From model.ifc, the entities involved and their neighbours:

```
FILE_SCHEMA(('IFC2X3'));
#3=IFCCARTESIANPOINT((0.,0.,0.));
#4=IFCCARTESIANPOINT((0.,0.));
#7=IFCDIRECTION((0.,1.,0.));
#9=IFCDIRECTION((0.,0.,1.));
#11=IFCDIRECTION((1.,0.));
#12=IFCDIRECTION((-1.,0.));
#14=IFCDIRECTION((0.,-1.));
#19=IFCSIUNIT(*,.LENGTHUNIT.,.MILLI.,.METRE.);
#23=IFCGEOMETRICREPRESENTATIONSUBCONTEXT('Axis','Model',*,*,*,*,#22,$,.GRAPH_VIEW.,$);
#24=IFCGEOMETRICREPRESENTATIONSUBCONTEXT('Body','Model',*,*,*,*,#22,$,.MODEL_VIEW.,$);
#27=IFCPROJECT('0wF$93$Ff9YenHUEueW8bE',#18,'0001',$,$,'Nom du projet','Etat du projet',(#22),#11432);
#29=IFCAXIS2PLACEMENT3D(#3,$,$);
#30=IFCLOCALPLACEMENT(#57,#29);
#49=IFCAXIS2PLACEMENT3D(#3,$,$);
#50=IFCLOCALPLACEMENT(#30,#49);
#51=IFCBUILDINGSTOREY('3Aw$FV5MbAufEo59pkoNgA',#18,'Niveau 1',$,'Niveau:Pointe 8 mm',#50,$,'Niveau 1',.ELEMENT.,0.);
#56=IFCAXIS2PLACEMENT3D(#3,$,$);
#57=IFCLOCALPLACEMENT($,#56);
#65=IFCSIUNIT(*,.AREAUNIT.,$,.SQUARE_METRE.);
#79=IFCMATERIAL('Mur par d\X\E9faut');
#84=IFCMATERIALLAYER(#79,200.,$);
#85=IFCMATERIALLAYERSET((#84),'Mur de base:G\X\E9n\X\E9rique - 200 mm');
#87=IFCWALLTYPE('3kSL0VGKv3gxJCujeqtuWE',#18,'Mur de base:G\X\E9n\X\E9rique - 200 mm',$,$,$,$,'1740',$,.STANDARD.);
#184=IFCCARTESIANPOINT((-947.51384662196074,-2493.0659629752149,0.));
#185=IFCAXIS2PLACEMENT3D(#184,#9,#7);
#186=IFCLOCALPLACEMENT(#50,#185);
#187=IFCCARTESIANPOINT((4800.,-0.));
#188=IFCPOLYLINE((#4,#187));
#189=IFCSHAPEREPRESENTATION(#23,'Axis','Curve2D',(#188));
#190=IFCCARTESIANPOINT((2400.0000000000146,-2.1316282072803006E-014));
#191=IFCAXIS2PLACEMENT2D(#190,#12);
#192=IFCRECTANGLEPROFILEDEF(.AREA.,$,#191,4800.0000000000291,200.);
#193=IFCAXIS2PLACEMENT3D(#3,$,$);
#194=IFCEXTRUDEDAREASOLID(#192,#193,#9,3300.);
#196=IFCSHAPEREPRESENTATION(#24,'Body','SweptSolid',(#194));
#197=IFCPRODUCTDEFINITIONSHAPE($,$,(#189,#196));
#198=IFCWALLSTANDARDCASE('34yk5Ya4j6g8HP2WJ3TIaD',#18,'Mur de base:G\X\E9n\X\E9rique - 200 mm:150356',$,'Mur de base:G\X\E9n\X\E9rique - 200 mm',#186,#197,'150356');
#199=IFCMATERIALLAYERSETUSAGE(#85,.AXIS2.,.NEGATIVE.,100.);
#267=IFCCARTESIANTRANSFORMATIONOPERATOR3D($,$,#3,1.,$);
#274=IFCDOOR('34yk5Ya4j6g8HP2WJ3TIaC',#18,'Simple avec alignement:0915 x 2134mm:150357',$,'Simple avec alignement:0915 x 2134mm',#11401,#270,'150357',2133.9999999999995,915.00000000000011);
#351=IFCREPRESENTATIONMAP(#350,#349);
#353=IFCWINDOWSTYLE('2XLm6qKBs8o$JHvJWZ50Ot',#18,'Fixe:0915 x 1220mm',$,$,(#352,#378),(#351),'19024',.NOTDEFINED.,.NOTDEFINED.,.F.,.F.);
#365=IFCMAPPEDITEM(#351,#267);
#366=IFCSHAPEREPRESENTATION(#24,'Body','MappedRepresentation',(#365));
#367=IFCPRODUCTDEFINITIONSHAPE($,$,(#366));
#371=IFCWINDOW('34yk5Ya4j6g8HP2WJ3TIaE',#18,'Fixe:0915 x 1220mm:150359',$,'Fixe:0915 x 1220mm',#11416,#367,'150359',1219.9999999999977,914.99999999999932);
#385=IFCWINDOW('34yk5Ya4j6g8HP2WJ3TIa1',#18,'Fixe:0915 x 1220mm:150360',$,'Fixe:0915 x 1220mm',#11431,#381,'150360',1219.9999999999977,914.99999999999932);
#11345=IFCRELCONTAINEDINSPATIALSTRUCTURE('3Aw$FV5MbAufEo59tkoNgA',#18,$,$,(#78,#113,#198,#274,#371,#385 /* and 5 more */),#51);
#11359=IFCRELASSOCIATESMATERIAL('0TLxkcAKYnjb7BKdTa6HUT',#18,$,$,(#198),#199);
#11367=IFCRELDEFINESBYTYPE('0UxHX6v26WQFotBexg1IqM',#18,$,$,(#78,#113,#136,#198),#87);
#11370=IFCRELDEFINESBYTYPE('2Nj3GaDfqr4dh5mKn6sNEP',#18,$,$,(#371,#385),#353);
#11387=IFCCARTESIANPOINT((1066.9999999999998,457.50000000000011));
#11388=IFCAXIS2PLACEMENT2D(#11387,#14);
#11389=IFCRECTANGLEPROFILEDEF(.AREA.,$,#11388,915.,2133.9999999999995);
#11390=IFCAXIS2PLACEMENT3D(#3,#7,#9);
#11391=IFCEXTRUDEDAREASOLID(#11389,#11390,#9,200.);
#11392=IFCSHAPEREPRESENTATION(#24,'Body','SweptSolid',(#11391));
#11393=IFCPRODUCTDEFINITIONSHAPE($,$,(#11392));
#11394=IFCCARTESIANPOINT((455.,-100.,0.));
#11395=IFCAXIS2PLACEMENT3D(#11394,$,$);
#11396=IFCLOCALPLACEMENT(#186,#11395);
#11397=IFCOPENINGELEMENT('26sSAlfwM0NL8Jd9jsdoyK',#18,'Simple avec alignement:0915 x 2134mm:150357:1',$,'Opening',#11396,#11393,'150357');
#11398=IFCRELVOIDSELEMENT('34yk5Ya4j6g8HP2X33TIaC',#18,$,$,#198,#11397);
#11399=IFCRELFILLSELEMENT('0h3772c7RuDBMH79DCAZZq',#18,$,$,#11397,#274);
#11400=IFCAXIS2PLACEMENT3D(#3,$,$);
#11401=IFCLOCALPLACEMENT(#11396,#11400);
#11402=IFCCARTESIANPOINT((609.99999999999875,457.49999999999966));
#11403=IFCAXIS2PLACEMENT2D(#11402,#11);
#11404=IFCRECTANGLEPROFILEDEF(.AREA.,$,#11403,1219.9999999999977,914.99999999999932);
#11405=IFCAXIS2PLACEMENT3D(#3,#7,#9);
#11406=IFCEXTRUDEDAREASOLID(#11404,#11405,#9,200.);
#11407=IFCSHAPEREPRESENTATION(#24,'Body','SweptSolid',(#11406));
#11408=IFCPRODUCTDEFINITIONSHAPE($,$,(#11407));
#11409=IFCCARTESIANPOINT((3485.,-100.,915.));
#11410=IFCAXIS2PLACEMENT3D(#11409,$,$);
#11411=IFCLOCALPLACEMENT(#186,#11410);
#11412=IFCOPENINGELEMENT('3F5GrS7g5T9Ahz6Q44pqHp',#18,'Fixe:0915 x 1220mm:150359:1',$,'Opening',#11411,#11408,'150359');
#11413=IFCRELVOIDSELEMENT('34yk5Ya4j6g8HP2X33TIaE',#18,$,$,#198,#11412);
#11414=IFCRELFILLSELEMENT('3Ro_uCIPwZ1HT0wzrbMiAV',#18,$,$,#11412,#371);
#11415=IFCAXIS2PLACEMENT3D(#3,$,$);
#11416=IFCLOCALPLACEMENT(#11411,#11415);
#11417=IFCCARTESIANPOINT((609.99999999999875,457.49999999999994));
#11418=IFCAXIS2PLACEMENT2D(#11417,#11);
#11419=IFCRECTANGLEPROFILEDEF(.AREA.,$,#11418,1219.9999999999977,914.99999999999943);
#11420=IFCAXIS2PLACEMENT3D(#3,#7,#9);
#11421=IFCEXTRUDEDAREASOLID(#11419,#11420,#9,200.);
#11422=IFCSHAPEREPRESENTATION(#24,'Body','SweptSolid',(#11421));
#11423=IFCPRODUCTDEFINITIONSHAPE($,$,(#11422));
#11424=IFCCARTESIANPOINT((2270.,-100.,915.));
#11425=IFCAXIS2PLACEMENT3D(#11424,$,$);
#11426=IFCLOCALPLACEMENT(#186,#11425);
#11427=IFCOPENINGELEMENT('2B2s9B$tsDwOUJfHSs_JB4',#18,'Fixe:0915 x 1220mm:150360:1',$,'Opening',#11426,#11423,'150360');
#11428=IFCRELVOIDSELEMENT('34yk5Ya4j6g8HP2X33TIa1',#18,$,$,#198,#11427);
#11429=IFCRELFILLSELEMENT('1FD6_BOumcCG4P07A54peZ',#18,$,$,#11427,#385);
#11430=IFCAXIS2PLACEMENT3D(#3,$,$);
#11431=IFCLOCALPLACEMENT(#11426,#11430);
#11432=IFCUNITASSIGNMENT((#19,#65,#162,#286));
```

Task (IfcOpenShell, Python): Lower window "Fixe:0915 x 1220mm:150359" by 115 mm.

```python
import numpy as np
import ifcopenshell
import ifcopenshell.api.geometry
import ifcopenshell.util.placement
import ifcopenshell.util.unit

model = ifcopenshell.open("model.ifc")
unit_scale = ifcopenshell.util.unit.calculate_unit_scale(model)

window = model.by_id(371)
opening = window.FillsVoids[0].RelatingOpeningElement
dz = -0.115 / unit_scale

shift = np.array([0.0, 0.0, dz])
# The window is placed relative to its opening, so it follows when the opening moves.
matrix = ifcopenshell.util.placement.get_local_placement(opening.ObjectPlacement)
matrix[:3, 3] += shift
ifcopenshell.api.geometry.edit_object_placement(
    model, product=opening, matrix=matrix, is_si=False, should_transform_children=True
)

print(f"moved by {dz * unit_scale:+.3f} m")

model.write("model-out.ifc")
```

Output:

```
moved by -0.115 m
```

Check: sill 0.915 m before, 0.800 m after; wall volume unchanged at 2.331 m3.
